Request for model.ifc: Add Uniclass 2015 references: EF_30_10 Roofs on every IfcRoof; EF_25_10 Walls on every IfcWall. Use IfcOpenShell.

First a look at what the model holds.

```python
import ifcopenshell

model = ifcopenshell.open("model.ifc")
print(model.schema)
print("classifications:", [c.Name for c in model.by_type("IfcClassification")])
for ifc_class in ("IfcDoor", "IfcRoof", "IfcStair", "IfcWall", "IfcWindow"):
    print(ifc_class, len(model.by_type(ifc_class)))
```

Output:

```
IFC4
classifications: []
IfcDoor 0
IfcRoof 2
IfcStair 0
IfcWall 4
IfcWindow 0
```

```python
import ifcopenshell
import ifcopenshell.api.classification

model = ifcopenshell.open("model.ifc")

system = ifcopenshell.api.classification.add_classification(model, classification="Uniclass 2015")

codes = {
    "IfcRoof": ("EF_30_10", "Roofs"),
    "IfcWall": ("EF_25_10", "Walls"),
}
for ifc_class, (code, name) in codes.items():
    products = model.by_type(ifc_class)
    ifcopenshell.api.classification.add_reference(
        model, products=products, classification=system, identification=code, name=name
    )
    print(code, len(products))

model.write("model_v2.ifc")
```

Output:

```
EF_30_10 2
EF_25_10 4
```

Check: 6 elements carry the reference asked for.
